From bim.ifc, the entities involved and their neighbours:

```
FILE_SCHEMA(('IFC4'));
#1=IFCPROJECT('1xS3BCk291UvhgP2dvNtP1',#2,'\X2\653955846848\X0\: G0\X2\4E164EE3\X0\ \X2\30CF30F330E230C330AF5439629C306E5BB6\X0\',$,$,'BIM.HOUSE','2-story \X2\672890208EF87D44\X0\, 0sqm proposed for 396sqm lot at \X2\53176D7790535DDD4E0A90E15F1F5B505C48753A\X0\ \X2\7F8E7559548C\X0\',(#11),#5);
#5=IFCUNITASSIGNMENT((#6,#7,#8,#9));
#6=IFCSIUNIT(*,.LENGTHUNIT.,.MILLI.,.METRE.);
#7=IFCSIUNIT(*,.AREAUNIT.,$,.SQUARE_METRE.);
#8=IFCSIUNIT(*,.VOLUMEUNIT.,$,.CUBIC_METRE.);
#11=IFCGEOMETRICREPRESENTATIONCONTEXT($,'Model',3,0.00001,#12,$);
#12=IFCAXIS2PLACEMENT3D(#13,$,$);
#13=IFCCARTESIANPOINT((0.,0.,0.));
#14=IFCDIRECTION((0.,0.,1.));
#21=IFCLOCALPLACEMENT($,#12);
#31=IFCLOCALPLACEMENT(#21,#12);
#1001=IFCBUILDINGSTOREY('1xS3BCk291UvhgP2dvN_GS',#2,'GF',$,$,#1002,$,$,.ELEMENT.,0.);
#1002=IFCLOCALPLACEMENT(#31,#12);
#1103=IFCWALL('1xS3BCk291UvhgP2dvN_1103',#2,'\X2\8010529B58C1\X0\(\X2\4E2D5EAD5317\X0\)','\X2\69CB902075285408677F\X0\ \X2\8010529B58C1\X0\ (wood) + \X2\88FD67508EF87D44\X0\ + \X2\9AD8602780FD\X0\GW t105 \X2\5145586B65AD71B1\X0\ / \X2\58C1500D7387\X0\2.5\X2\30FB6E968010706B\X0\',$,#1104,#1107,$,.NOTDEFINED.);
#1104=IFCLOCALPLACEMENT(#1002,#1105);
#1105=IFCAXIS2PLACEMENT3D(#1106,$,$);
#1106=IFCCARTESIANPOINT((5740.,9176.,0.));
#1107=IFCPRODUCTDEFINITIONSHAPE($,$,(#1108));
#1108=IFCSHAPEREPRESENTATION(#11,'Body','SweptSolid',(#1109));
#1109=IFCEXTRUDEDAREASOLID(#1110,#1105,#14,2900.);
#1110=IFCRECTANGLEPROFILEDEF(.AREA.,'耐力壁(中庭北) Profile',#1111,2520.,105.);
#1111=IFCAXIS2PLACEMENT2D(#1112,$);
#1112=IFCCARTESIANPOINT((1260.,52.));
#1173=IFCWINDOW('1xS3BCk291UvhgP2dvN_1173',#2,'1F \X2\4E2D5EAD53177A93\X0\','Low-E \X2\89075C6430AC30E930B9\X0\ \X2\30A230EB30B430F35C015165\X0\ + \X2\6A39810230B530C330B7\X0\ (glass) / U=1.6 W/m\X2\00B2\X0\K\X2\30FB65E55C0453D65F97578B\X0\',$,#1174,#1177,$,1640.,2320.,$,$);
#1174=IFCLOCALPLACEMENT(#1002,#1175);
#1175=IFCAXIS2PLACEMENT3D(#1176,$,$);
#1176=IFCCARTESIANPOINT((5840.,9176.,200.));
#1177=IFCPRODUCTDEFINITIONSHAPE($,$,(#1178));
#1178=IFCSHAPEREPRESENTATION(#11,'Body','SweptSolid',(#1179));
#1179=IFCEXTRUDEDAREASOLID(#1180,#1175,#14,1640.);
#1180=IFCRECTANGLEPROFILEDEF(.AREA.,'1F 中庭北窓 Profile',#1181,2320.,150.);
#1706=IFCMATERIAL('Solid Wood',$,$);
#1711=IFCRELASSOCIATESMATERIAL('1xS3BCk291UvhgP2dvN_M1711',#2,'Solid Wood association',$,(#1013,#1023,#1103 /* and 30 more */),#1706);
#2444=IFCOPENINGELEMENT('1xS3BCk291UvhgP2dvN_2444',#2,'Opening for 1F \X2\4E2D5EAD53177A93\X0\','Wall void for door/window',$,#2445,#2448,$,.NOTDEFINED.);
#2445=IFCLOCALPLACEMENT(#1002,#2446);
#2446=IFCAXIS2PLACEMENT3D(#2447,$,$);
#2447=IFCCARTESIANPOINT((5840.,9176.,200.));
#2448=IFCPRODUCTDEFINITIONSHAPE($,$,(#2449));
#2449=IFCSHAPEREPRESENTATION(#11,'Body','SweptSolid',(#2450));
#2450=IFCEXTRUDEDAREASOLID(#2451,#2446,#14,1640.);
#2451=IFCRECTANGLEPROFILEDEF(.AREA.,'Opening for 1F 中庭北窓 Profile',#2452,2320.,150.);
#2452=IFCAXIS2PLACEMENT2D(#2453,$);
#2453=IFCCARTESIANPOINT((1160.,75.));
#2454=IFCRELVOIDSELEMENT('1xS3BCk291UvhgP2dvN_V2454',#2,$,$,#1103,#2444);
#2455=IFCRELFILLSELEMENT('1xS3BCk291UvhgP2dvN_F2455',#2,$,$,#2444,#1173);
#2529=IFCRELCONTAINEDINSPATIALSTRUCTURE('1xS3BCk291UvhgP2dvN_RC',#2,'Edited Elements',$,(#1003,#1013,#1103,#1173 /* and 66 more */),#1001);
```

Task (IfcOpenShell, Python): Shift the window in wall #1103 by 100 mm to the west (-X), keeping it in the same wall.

```python
import ifcopenshell
import ifcopenshell.api.geometry
import ifcopenshell.util.placement
import ifcopenshell.util.unit

model = ifcopenshell.open("bim.ifc")
unit_scale = ifcopenshell.util.unit.calculate_unit_scale(model)

window = model.by_guid("1xS3BCk291UvhgP2dvN_1173")
opening = window.FillsVoids[0].RelatingOpeningElement
wall = opening.VoidsElements[0].RelatingBuildingElement

wall_matrix = ifcopenshell.util.placement.get_local_placement(wall.ObjectPlacement)
shift = wall_matrix[:3, 0] * -0.1 / unit_scale
before = ifcopenshell.util.placement.get_local_placement(window.ObjectPlacement)[:3, 3].copy()

# The window is not placed relative to its opening, so move both.
for product in (opening, window):
    matrix = ifcopenshell.util.placement.get_local_placement(product.ObjectPlacement)
    matrix[:3, 3] += shift
    ifcopenshell.api.geometry.edit_object_placement(model, product=product, matrix=matrix, is_si=False)

after = ifcopenshell.util.placement.get_local_placement(window.ObjectPlacement)[:3, 3]
print("window moved by", (after - before).round(3) + 0.0)

model.write("bim_rev.ifc")
```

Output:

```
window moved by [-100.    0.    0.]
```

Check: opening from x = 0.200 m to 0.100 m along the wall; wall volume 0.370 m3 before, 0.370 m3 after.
